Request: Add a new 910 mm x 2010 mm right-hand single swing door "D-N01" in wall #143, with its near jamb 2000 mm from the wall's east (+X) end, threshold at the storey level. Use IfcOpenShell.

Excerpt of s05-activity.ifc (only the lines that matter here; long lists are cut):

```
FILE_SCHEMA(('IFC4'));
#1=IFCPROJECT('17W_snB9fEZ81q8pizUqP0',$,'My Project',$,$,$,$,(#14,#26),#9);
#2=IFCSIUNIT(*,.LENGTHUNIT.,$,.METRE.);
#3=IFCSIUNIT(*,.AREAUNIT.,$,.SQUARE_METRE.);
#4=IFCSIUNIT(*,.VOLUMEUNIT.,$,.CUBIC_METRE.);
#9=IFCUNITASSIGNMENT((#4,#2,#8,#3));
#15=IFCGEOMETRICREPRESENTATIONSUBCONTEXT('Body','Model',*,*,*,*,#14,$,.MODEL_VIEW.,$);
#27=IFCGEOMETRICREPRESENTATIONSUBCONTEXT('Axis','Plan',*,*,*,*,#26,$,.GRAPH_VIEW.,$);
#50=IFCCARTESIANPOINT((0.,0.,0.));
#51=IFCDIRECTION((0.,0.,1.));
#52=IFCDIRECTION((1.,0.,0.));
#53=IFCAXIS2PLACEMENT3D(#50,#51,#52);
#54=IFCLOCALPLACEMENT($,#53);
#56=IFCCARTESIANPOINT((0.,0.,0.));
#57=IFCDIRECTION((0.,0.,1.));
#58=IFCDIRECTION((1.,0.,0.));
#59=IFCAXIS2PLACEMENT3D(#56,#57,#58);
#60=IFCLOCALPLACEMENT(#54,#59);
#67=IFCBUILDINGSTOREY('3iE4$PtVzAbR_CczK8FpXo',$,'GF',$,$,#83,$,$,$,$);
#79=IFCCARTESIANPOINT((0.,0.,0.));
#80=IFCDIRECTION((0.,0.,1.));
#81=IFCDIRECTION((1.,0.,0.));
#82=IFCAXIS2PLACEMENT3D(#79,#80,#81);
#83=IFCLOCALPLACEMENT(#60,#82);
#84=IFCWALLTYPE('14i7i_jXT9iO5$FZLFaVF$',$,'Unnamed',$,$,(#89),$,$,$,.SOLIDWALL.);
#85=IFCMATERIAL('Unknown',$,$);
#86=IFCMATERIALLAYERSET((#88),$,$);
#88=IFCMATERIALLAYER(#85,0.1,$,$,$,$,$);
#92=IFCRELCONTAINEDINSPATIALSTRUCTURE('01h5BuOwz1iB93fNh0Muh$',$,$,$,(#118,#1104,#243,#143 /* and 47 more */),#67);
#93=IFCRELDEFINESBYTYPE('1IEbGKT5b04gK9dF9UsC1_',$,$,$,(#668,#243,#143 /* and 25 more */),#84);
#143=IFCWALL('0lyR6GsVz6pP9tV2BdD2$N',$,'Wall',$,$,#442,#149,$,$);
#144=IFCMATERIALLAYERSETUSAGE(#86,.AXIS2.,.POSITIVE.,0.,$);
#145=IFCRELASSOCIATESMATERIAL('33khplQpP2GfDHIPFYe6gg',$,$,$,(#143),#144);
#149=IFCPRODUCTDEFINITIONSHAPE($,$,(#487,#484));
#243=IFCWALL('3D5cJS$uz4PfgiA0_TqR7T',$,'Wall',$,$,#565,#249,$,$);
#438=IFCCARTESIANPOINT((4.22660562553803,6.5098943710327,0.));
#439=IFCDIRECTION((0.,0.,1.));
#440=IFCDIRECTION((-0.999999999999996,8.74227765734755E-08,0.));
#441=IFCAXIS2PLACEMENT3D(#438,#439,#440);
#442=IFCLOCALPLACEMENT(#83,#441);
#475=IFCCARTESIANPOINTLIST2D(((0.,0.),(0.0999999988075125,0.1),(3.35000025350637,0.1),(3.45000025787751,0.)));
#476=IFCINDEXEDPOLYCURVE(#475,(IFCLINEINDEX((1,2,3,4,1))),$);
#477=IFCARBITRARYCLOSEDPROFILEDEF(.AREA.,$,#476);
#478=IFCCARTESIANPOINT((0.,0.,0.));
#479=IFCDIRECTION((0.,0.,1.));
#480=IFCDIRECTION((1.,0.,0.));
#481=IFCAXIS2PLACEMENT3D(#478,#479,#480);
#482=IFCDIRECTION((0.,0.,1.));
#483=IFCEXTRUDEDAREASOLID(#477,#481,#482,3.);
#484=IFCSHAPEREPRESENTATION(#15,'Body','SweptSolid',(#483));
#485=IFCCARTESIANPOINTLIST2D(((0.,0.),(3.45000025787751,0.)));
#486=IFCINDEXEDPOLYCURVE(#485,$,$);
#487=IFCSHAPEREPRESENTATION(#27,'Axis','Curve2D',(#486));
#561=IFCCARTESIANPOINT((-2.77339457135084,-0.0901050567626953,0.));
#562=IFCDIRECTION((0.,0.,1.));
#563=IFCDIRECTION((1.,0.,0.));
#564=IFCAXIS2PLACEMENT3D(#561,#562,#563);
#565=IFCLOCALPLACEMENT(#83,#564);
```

```python
import numpy as np
import ifcopenshell
import ifcopenshell.api.feature
import ifcopenshell.api.geometry
import ifcopenshell.api.root
import ifcopenshell.api.spatial
import ifcopenshell.geom
import ifcopenshell.util.element
import ifcopenshell.util.placement
import ifcopenshell.util.representation
import ifcopenshell.util.shape
import ifcopenshell.util.unit

model = ifcopenshell.open("s05-activity.ifc")
unit_scale = ifcopenshell.util.unit.calculate_unit_scale(model)
settings = ifcopenshell.geom.settings()


def volume(element):
    """Net volume in cubic metres, openings subtracted."""
    shape = ifcopenshell.geom.create_shape(settings, element)
    return ifcopenshell.util.shape.get_volume(shape.geometry)


wall = model.by_guid("0lyR6GsVz6pP9tV2BdD2$N")
storey = ifcopenshell.util.element.get_container(wall, ifc_class="IfcBuildingStorey")
context = ifcopenshell.util.representation.get_context(model, "Model", "Body", "MODEL_VIEW")
before = volume(wall)

width, height, from_end, sill = 0.91, 2.01, 2, 0.0  # metres

# The wall runs along its own X axis, and the end named is its -X end.
wall_shape = ifcopenshell.geom.create_shape(settings, wall)
x, y, z = ifcopenshell.util.shape.get_vertices(wall_shape.geometry).T
start = x.min() + from_end
face, thickness = float(y.min()), float(y.max() - y.min())
wall_matrix = ifcopenshell.util.placement.get_local_placement(wall.ObjectPlacement)
level = ifcopenshell.util.placement.get_local_placement(storey.ObjectPlacement)[2, 3]


def in_wall(x, y):
    """Placement at x, y metres in the wall's axes, at sill height."""
    matrix = wall_matrix.copy()
    matrix[:, 3] = wall_matrix @ np.array([x / unit_scale, y / unit_scale, 0.0, 1.0])
    matrix[2, 3] = level + sill / unit_scale
    return matrix


# Opening: a box that overshoots both wall faces by 50 mm.
opening = ifcopenshell.api.root.create_entity(model, ifc_class="IfcOpeningElement", predefined_type="OPENING")
box = ifcopenshell.api.geometry.add_wall_representation(
    model, context=context, length=width, height=height, thickness=thickness + 0.1
)
ifcopenshell.api.geometry.assign_representation(model, product=opening, representation=box)
ifcopenshell.api.geometry.edit_object_placement(model, product=opening, matrix=in_wall(start, face - 0.05), is_si=False)
ifcopenshell.api.feature.add_feature(model, feature=opening, element=wall)

door = ifcopenshell.api.root.create_entity(model, ifc_class="IfcDoor", name="D-N01", predefined_type="DOOR")
door.OverallWidth, door.OverallHeight = width / unit_scale, height / unit_scale
door.OperationType = "SINGLE_SWING_RIGHT"
body = ifcopenshell.api.geometry.add_door_representation(
    model,
    context=context,
    overall_width=door.OverallWidth,
    overall_height=door.OverallHeight,
    operation_type="SINGLE_SWING_RIGHT",
    lining_properties={"LiningDepth": thickness / unit_scale, "ThresholdDepth": thickness / unit_scale},
)
ifcopenshell.api.geometry.assign_representation(model, product=door, representation=body)
ifcopenshell.api.spatial.assign_container(model, products=[door], relating_structure=storey)
ifcopenshell.api.feature.add_filling(model, opening=opening, element=door)

# The lining spans the wall, so the door starts at the wall face.
ifcopenshell.api.geometry.edit_object_placement(model, product=door, matrix=in_wall(start, face), is_si=False)

after = volume(wall)

print(f"wall volume {before:.3f} -> {after:.3f} m3")

model.write("s05-activity_edited.ifc")
```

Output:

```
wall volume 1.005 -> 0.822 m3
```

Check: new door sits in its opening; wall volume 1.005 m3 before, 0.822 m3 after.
